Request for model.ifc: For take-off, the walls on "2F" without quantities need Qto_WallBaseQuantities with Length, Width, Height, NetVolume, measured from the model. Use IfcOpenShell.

First a look at what the model holds.

```python
import ifcopenshell
import ifcopenshell.util.element
import ifcopenshell.util.unit

model = ifcopenshell.open("model.ifc")
print(model.schema)
for unit_type in ("LENGTHUNIT", "AREAUNIT", "VOLUMEUNIT"):
    print(unit_type, ifcopenshell.util.unit.calculate_unit_scale(model, unit_type))
storey = next(s for s in model.by_type("IfcBuildingStorey") if s.Name == "2F")
walls = [e for e in ifcopenshell.util.element.get_decomposition(storey) if e.is_a("IfcWall")]
for e in sorted(walls, key=lambda e: e.id()):
    print(e.id(), e.is_a(), e.Name, list(ifcopenshell.util.element.get_psets(e, qtos_only=True)), sep=" | ")
```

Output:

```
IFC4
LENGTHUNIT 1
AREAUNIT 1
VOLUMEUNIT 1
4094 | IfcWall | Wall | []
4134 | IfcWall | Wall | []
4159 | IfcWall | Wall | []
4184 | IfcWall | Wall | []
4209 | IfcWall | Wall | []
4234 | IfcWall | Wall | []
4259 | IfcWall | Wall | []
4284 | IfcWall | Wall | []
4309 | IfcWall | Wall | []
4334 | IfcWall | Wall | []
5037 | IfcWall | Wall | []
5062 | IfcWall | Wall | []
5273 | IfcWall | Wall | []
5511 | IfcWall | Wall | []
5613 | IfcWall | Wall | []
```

```python
import ifcopenshell
import ifcopenshell.api.pset
import ifcopenshell.geom
import ifcopenshell.util.element
import ifcopenshell.util.shape
import ifcopenshell.util.unit

model = ifcopenshell.open("model.ifc")
unit_scale = ifcopenshell.util.unit.calculate_unit_scale(model)
volume_scale = ifcopenshell.util.unit.calculate_unit_scale(model, "VOLUMEUNIT")
settings = ifcopenshell.geom.settings()

storey = next(s for s in model.by_type("IfcBuildingStorey") if s.Name == "2F")
walls = [e for e in ifcopenshell.util.element.get_decomposition(storey) if e.is_a("IfcWall")]

for e in sorted(walls, key=lambda e: e.id()):
    if ifcopenshell.util.element.get_psets(e, qtos_only=True, should_inherit=False):
        continue
    # Geometry comes back in metres, in the element's own axes.
    shape = ifcopenshell.geom.create_shape(settings, e)
    values = {
        "Length": ifcopenshell.util.shape.get_x(shape.geometry) / unit_scale,
        "Width": ifcopenshell.util.shape.get_y(shape.geometry) / unit_scale,
        "Height": ifcopenshell.util.shape.get_z(shape.geometry) / unit_scale,
        "NetVolume": ifcopenshell.util.shape.get_volume(shape.geometry) / volume_scale,
    }
    qto = ifcopenshell.api.pset.add_qto(model, product=e, name="Qto_WallBaseQuantities")
    ifcopenshell.api.pset.edit_qto(model, qto=qto, properties=values)
    print(e.id(), {k: round(v, 3) for k, v in values.items()})

model.write("model_rev.ifc")
```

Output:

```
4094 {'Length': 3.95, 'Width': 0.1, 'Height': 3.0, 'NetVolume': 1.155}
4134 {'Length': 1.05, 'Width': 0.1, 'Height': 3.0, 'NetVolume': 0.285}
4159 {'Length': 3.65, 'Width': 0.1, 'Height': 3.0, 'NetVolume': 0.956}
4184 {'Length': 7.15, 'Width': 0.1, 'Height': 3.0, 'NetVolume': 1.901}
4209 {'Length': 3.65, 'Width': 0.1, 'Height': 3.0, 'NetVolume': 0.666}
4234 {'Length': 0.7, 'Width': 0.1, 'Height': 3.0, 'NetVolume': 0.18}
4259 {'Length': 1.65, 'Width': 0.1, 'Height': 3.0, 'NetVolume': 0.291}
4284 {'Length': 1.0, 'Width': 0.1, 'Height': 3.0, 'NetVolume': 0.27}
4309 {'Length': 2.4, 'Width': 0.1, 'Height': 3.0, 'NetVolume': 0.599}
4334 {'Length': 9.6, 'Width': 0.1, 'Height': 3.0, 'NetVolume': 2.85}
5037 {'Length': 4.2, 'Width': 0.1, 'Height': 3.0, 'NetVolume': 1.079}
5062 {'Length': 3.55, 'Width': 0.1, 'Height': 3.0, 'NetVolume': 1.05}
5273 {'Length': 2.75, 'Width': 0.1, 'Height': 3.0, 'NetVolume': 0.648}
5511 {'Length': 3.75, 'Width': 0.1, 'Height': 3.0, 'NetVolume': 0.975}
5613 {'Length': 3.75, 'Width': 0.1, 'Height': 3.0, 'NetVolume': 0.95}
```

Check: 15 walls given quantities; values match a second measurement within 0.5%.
